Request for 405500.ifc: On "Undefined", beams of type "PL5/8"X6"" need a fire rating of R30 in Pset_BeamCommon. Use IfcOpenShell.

First a look at what the model holds.

```python
import ifcopenshell
import ifcopenshell.util.element

model = ifcopenshell.open("405500.ifc")
print(model.schema)
storey = next(s for s in model.by_type("IfcBuildingStorey") if s.Name == "Undefined")
beams = [e for e in ifcopenshell.util.element.get_decomposition(storey) if e.is_a("IfcBeam")]
seen = {}
for e in beams:
    element_type = ifcopenshell.util.element.get_type(e)
    key = (element_type.Name if element_type != e and element_type else None, ifcopenshell.util.element.get_pset(e, "Pset_BeamCommon", "FireRating"))
    seen[key] = seen.get(key, 0) + 1
for (name, value), count in sorted(seen.items(), key=str):
    print(count, "x", name, "|", value)
```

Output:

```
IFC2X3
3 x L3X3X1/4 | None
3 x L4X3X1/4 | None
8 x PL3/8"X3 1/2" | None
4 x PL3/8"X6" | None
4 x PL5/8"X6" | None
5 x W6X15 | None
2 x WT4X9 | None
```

```python
import ifcopenshell
import ifcopenshell.api.pset
import ifcopenshell.util.element

model = ifcopenshell.open("405500.ifc")

storey = next(s for s in model.by_type("IfcBuildingStorey") if s.Name == "Undefined")
beams = [e for e in ifcopenshell.util.element.get_decomposition(storey) if e.is_a("IfcBeam")]

count = 0
for e in beams:
    element_type = ifcopenshell.util.element.get_type(e)
    if element_type in (None, e) or element_type.Name != 'PL5/8"X6"':
        continue
    found = ifcopenshell.util.element.get_pset(e, "Pset_BeamCommon", should_inherit=False)
    if found:
        pset = model.by_id(found["id"])
        if len(ifcopenshell.util.element.get_elements_by_pset(pset)) > 1:
            pset = ifcopenshell.api.pset.unshare_pset(model, products=[e], pset=pset)[0]
    else:
        pset = ifcopenshell.api.pset.add_pset(model, product=e, name="Pset_BeamCommon")
    ifcopenshell.api.pset.edit_pset(model, pset=pset, properties={"FireRating": "R30"})
    count += 1

print(count, "beams updated")

model.write("405500_v2.ifc")
```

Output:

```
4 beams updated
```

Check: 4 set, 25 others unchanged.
